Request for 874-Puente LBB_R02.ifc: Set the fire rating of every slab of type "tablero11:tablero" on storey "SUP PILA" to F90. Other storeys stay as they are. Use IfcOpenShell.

First a look at what the model holds.

```python
import ifcopenshell
import ifcopenshell.util.element

model = ifcopenshell.open("874-Puente LBB_R02.ifc")
print(model.schema)
storey = next(s for s in model.by_type("IfcBuildingStorey") if s.Name == "SUP PILA")
slabs = [e for e in ifcopenshell.util.element.get_decomposition(storey) if e.is_a("IfcSlab")]
seen = {}
for e in slabs:
    element_type = ifcopenshell.util.element.get_type(e)
    key = (element_type.Name if element_type != e and element_type else None, ifcopenshell.util.element.get_pset(e, "Pset_SlabCommon", "FireRating"))
    seen[key] = seen.get(key, 0) + 1
for (name, value), count in sorted(seen.items(), key=str):
    print(count, "x", name, "|", value)
```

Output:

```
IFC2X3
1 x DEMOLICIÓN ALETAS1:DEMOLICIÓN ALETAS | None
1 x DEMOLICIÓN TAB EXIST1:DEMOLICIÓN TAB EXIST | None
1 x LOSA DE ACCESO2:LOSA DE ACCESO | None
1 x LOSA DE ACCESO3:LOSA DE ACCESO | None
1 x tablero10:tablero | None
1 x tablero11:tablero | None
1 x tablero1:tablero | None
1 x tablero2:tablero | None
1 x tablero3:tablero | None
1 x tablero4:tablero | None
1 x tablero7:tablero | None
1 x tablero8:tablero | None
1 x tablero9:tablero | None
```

```python
import ifcopenshell
import ifcopenshell.api.pset
import ifcopenshell.util.element

model = ifcopenshell.open("874-Puente LBB_R02.ifc")

storey = next(s for s in model.by_type("IfcBuildingStorey") if s.Name == "SUP PILA")
slabs = [e for e in ifcopenshell.util.element.get_decomposition(storey) if e.is_a("IfcSlab")]

count = 0
for e in slabs:
    element_type = ifcopenshell.util.element.get_type(e)
    if element_type in (None, e) or element_type.Name != "tablero11:tablero":
        continue
    # add_pset returns the element's existing set when there is one.
    pset = ifcopenshell.api.pset.add_pset(model, product=e, name="Pset_SlabCommon")
    ifcopenshell.api.pset.edit_pset(model, pset=pset, properties={"FireRating": "F90"})
    count += 1

print(count, "slabs updated")

model.write("874-Puente LBB_R02_updated.ifc")
```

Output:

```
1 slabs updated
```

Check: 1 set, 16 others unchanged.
